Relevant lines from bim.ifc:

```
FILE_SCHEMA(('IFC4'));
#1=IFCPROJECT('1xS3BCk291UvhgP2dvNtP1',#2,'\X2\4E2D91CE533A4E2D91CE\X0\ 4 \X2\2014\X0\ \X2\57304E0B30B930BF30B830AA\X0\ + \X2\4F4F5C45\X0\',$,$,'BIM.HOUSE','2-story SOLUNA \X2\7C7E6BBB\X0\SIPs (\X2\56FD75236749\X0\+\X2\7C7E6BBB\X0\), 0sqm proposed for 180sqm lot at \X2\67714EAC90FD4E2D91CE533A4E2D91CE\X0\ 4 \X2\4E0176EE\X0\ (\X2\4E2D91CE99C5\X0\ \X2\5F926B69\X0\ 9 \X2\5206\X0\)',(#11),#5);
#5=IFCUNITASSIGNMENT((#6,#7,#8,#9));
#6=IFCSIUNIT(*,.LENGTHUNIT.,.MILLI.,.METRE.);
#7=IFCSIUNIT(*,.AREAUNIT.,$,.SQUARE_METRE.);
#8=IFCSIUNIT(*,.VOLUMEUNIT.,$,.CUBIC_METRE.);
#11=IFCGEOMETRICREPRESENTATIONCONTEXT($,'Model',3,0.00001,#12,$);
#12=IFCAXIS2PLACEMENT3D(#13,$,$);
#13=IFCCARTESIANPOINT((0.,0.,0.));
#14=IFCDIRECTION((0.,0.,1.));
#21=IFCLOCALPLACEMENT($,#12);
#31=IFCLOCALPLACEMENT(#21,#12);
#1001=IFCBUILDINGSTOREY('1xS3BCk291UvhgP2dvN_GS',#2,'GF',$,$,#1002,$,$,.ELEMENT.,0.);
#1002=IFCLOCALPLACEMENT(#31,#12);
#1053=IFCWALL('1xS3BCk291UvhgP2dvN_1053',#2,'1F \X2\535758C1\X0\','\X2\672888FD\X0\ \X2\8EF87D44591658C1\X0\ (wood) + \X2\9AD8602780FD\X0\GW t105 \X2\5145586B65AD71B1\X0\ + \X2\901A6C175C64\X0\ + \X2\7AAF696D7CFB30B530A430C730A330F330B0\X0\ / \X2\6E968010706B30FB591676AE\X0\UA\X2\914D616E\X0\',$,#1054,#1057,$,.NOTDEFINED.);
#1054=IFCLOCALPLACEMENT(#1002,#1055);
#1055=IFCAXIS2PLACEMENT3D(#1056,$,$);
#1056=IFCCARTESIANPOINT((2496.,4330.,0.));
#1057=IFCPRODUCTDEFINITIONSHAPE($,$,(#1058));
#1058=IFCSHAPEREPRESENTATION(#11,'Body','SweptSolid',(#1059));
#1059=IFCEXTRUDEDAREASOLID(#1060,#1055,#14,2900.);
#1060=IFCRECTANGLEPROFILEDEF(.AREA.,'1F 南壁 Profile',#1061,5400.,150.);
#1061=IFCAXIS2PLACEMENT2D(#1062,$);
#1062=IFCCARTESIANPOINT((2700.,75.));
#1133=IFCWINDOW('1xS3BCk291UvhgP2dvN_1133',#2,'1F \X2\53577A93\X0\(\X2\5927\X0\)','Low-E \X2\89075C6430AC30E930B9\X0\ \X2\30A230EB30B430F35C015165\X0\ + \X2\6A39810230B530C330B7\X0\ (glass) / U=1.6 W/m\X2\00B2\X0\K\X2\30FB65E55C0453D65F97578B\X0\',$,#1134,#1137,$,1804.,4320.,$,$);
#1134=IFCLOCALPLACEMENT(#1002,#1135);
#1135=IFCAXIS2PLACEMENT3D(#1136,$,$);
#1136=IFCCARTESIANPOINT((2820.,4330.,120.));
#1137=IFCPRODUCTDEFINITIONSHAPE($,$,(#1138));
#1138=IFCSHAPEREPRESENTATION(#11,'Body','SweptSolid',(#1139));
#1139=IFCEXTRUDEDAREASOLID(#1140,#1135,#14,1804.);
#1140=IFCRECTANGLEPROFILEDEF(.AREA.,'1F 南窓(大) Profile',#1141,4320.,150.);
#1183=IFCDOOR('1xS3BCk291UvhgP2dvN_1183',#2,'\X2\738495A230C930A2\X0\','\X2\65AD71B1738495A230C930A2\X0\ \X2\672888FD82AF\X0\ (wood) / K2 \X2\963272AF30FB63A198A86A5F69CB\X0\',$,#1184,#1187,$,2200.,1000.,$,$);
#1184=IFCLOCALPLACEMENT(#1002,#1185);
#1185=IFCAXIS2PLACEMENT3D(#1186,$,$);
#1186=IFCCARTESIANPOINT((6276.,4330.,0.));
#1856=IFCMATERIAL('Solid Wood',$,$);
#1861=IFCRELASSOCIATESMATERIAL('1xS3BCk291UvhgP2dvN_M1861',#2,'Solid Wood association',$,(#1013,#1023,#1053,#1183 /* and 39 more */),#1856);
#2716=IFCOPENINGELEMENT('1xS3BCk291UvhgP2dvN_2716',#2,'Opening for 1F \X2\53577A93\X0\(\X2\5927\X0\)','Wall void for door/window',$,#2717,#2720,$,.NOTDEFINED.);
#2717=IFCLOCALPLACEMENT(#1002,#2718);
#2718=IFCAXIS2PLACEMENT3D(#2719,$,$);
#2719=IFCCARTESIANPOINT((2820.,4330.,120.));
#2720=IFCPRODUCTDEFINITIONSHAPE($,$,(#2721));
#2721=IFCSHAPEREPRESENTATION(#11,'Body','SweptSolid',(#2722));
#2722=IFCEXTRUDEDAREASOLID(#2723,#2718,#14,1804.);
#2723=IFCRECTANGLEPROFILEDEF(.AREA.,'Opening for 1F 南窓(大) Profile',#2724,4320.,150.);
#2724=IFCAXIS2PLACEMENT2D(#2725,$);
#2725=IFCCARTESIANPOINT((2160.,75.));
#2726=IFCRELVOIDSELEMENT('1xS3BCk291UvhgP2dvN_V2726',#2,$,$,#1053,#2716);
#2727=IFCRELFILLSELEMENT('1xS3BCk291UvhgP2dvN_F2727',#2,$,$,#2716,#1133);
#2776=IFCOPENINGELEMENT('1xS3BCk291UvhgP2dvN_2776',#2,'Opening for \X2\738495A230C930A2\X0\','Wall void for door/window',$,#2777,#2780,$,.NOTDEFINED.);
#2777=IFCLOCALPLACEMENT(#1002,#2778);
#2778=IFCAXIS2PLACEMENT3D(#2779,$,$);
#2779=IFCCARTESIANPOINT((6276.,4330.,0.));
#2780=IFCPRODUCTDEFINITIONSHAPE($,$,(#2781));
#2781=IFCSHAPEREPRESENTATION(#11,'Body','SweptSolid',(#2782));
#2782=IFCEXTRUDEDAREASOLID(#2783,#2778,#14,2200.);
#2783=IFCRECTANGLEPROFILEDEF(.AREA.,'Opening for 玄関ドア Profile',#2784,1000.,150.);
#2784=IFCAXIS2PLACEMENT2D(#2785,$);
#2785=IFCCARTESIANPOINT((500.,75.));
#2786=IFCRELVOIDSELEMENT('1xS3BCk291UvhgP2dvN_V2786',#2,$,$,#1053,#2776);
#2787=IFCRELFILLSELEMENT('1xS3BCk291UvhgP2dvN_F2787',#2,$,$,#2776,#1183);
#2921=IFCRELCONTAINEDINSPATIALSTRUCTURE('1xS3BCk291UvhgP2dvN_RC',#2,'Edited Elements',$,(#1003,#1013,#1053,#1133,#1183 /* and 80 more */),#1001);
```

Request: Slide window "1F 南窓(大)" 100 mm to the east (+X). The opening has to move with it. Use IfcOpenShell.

```python
import ifcopenshell
import ifcopenshell.api.geometry
import ifcopenshell.util.placement

model = ifcopenshell.open("bim.ifc")

window = model.by_id(1133)
opening = window.FillsVoids[0].RelatingOpeningElement
wall = opening.VoidsElements[0].RelatingBuildingElement

wall_matrix = ifcopenshell.util.placement.get_local_placement(wall.ObjectPlacement)
shift = wall_matrix[:3, 0] * 100.0
before = ifcopenshell.util.placement.get_local_placement(window.ObjectPlacement)[:3, 3].copy()

# The window is not placed relative to its opening, so move both.
for product in (opening, window):
    matrix = ifcopenshell.util.placement.get_local_placement(product.ObjectPlacement)
    matrix[:3, 3] += shift
    ifcopenshell.api.geometry.edit_object_placement(model, product=product, matrix=matrix, is_si=False)

after = ifcopenshell.util.placement.get_local_placement(window.ObjectPlacement)[:3, 3]
print("window moved by", (after - before).round(3) + 0.0)

model.write("bim_updated.ifc")
```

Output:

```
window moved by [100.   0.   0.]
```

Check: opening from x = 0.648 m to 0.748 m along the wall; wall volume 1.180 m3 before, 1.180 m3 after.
